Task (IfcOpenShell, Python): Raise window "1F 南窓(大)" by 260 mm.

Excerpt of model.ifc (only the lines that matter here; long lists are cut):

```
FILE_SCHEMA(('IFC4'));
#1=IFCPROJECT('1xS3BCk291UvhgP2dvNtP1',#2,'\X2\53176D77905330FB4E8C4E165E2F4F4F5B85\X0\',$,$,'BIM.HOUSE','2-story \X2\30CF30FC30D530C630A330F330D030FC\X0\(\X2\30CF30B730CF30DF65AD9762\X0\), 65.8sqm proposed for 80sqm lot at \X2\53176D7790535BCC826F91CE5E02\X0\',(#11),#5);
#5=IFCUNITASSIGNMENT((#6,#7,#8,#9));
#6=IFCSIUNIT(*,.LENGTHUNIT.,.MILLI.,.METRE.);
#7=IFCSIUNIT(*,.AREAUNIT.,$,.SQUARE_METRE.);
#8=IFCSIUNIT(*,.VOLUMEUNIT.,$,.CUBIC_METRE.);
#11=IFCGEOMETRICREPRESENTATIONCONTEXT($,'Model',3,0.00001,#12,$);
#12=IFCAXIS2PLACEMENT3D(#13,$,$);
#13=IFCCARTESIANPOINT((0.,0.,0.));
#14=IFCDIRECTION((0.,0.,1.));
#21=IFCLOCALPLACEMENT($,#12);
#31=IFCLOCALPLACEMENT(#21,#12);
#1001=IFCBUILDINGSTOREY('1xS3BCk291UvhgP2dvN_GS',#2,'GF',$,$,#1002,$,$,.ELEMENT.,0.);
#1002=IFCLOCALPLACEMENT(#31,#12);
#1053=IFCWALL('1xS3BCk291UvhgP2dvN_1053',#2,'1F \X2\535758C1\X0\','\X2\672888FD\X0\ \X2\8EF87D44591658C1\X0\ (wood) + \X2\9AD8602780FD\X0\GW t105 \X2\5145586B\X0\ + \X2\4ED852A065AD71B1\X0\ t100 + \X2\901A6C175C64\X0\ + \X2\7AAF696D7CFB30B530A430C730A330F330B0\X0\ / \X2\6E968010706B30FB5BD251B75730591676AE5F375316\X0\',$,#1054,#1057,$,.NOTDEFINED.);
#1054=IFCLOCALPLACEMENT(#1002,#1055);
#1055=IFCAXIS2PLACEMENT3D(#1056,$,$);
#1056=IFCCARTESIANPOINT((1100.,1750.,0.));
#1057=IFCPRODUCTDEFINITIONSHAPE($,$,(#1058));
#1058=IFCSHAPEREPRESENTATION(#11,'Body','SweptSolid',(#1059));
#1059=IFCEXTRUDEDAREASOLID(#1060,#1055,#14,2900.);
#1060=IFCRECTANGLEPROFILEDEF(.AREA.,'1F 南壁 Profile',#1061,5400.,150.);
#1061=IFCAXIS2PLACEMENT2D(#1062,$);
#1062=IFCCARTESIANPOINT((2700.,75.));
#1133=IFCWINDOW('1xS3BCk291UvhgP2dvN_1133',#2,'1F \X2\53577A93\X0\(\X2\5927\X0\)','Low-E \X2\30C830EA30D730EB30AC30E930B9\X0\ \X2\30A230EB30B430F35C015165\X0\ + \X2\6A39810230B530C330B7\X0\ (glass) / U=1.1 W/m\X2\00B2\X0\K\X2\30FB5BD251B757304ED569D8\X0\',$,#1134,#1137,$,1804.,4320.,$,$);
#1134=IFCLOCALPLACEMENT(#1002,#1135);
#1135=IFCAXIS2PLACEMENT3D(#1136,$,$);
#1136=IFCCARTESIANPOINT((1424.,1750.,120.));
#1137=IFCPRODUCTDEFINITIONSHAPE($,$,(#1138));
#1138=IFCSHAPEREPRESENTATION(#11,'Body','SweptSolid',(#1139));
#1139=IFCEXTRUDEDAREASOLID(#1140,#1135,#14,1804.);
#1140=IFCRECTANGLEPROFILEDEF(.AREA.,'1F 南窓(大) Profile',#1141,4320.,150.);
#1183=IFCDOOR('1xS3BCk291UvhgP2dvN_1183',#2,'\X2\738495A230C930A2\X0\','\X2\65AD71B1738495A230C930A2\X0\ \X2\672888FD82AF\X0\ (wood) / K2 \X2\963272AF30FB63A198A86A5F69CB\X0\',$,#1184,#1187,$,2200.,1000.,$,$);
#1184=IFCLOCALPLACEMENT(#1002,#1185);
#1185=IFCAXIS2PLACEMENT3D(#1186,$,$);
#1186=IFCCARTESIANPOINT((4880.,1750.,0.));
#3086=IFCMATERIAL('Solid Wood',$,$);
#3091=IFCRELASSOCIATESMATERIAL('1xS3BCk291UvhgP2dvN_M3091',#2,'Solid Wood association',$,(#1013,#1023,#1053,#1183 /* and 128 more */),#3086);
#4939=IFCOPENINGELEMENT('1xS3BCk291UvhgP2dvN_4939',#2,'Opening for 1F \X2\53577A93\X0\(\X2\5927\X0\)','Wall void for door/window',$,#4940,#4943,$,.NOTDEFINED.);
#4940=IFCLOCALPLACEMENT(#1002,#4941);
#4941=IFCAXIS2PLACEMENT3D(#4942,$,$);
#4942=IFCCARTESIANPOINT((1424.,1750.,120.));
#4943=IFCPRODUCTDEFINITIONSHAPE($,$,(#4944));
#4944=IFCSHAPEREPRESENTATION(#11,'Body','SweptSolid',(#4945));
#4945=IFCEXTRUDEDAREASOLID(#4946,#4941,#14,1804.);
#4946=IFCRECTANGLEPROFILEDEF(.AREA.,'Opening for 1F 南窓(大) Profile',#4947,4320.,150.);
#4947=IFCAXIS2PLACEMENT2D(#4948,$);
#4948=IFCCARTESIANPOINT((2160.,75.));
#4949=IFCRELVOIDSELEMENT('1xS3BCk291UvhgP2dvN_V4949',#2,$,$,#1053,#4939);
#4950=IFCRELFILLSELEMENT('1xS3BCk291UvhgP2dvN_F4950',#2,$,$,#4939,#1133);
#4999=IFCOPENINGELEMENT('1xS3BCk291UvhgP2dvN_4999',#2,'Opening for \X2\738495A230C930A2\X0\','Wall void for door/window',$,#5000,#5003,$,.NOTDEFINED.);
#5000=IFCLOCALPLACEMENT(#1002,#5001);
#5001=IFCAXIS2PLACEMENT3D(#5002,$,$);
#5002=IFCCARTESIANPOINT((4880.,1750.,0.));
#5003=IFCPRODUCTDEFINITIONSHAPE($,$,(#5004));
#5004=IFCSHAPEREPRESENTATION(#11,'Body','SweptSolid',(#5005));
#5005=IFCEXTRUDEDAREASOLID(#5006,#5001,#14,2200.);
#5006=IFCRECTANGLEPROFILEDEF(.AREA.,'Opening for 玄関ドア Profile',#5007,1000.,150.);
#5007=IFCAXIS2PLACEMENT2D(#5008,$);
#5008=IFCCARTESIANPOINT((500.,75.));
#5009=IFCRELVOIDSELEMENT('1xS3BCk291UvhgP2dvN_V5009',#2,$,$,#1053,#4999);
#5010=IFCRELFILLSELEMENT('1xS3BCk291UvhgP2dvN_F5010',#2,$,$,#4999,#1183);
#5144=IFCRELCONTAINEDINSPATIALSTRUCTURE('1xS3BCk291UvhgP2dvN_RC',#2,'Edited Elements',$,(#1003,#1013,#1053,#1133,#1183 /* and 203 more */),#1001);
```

```python
import numpy as np
import ifcopenshell
import ifcopenshell.api.geometry
import ifcopenshell.util.placement
import ifcopenshell.util.unit

model = ifcopenshell.open("model.ifc")
unit_scale = ifcopenshell.util.unit.calculate_unit_scale(model)

window = model.by_id(1133)
opening = window.FillsVoids[0].RelatingOpeningElement
dz = 0.26 / unit_scale

shift = np.array([0.0, 0.0, dz])
# The window is not placed relative to its opening, so move both.
for product in (opening, window):
    matrix = ifcopenshell.util.placement.get_local_placement(product.ObjectPlacement)
    matrix[:3, 3] += shift
    ifcopenshell.api.geometry.edit_object_placement(model, product=product, matrix=matrix, is_si=False)

print(f"moved by {dz * unit_scale:+.3f} m")

model.write("model-out.ifc")
```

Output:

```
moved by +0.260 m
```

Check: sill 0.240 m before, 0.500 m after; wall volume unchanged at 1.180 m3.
